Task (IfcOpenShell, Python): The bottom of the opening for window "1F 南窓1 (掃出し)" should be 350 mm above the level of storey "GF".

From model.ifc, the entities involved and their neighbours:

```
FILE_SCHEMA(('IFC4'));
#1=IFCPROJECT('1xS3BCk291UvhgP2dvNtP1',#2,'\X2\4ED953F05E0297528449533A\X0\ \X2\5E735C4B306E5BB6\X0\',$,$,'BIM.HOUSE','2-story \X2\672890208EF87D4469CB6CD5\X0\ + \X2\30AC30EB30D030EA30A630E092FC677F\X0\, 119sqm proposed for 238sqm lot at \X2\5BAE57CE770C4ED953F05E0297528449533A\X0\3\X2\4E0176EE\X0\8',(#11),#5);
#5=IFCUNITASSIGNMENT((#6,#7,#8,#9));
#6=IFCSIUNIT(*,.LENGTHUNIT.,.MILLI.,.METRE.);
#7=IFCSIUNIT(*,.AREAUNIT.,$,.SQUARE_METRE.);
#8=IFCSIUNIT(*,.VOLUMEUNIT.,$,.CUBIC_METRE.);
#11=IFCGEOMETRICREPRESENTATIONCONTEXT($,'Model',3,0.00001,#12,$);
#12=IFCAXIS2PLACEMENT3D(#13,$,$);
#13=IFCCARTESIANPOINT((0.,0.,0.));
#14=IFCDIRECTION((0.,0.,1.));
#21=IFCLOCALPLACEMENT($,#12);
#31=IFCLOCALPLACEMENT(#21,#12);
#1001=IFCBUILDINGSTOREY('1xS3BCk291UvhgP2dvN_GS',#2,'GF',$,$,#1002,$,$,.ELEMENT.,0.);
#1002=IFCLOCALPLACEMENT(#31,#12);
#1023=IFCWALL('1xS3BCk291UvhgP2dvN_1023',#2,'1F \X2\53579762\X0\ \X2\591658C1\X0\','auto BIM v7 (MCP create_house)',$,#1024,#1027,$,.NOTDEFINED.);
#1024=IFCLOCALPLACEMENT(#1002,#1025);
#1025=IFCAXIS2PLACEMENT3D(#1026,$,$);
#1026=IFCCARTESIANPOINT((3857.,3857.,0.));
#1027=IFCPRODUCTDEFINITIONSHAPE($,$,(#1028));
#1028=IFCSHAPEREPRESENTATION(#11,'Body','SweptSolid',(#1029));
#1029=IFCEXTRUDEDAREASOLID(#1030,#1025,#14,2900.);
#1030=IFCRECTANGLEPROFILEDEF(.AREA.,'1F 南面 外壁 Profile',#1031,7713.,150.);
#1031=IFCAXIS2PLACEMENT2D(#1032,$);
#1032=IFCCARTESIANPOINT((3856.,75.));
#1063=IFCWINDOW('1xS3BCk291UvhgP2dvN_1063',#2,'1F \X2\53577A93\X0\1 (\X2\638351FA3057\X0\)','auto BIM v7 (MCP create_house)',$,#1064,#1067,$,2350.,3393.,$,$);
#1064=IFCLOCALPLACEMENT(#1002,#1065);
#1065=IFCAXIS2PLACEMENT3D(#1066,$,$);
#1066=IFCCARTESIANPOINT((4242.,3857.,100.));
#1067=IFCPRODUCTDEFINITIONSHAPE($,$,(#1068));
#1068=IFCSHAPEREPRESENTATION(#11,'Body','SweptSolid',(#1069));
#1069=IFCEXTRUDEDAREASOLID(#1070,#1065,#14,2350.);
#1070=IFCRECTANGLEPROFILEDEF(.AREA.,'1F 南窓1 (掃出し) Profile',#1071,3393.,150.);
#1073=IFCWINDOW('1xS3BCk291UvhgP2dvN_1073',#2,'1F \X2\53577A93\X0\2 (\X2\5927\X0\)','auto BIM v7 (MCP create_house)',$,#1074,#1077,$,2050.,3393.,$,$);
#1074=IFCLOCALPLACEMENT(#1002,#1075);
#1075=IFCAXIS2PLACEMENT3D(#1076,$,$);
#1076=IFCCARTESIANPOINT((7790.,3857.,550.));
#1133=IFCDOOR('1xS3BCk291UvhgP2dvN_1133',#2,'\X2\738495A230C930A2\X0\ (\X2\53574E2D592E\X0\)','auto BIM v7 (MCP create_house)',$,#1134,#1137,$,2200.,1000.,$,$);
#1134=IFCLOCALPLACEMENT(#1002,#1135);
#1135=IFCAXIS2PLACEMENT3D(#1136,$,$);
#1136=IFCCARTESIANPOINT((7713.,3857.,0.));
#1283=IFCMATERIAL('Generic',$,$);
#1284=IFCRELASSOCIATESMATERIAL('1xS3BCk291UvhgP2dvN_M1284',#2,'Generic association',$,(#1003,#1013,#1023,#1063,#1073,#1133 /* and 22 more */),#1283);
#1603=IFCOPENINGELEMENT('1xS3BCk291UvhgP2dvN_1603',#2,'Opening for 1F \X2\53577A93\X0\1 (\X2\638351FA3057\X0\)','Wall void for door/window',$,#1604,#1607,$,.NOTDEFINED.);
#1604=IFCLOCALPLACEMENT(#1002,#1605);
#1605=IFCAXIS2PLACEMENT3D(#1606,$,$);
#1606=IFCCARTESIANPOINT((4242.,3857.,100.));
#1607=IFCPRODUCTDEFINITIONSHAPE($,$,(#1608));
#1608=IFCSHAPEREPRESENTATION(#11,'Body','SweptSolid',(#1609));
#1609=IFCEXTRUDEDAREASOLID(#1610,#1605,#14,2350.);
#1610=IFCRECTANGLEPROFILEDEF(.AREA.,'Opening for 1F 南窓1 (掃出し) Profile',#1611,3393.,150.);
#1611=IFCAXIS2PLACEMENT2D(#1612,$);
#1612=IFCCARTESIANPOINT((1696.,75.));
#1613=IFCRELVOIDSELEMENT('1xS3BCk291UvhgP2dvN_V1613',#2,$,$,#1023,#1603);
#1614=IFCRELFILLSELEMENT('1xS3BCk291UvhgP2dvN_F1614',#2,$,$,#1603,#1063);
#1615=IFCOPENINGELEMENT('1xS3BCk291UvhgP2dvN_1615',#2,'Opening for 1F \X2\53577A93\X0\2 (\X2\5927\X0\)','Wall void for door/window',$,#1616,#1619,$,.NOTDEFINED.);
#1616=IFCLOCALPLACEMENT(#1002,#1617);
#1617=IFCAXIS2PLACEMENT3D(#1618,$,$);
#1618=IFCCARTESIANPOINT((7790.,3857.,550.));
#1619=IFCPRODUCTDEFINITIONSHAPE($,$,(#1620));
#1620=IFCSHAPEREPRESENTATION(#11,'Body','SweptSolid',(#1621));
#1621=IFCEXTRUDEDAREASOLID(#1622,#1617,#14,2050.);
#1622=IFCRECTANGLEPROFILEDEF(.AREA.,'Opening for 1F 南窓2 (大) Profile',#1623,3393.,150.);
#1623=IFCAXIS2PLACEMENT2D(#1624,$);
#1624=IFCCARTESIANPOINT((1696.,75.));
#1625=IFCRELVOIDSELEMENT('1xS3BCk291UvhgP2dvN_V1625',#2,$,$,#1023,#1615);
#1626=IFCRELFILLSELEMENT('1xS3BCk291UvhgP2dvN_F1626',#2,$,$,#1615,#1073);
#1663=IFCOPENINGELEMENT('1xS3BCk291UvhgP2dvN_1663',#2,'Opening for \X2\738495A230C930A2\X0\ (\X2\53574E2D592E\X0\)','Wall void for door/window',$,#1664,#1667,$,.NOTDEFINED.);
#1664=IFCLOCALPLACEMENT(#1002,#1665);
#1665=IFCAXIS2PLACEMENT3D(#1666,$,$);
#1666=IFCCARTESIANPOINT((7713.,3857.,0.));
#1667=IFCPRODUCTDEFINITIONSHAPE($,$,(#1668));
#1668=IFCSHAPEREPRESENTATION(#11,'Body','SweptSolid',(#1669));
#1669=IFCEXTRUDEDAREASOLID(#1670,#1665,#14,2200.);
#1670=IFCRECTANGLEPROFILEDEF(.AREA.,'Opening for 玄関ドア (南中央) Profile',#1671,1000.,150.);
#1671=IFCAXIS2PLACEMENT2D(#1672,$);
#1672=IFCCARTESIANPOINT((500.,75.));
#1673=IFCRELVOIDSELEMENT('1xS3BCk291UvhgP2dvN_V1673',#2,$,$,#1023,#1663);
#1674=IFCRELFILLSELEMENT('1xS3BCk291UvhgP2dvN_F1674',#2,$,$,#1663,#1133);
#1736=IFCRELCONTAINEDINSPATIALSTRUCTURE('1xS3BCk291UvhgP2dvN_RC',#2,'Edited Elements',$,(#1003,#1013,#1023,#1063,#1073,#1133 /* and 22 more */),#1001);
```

```python
import numpy as np
import ifcopenshell
import ifcopenshell.api.geometry
import ifcopenshell.geom
import ifcopenshell.util.element
import ifcopenshell.util.placement
import ifcopenshell.util.shape
import ifcopenshell.util.unit

model = ifcopenshell.open("model.ifc")
unit_scale = ifcopenshell.util.unit.calculate_unit_scale(model)

window = model.by_id(1063)
opening = window.FillsVoids[0].RelatingOpeningElement
storey = ifcopenshell.util.element.get_container(window, ifc_class="IfcBuildingStorey")
level = ifcopenshell.util.placement.get_local_placement(storey.ObjectPlacement)[2, 3]

# The opening's origin need not be at the sill, so measure its lowest point.
shape = ifcopenshell.geom.create_shape(ifcopenshell.geom.settings(), opening)
bottom = ifcopenshell.util.shape.get_shape_bottom_elevation(shape, shape.geometry) / unit_scale
dz = level + 0.35 / unit_scale - bottom

shift = np.array([0.0, 0.0, dz])
# The window is not placed relative to its opening, so move both.
for product in (opening, window):
    matrix = ifcopenshell.util.placement.get_local_placement(product.ObjectPlacement)
    matrix[:3, 3] += shift
    ifcopenshell.api.geometry.edit_object_placement(model, product=product, matrix=matrix, is_si=False)

print(f"moved by {dz * unit_scale:+.3f} m")

model.write("model_updated.ifc")
```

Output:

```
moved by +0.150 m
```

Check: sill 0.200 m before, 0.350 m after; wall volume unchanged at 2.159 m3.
